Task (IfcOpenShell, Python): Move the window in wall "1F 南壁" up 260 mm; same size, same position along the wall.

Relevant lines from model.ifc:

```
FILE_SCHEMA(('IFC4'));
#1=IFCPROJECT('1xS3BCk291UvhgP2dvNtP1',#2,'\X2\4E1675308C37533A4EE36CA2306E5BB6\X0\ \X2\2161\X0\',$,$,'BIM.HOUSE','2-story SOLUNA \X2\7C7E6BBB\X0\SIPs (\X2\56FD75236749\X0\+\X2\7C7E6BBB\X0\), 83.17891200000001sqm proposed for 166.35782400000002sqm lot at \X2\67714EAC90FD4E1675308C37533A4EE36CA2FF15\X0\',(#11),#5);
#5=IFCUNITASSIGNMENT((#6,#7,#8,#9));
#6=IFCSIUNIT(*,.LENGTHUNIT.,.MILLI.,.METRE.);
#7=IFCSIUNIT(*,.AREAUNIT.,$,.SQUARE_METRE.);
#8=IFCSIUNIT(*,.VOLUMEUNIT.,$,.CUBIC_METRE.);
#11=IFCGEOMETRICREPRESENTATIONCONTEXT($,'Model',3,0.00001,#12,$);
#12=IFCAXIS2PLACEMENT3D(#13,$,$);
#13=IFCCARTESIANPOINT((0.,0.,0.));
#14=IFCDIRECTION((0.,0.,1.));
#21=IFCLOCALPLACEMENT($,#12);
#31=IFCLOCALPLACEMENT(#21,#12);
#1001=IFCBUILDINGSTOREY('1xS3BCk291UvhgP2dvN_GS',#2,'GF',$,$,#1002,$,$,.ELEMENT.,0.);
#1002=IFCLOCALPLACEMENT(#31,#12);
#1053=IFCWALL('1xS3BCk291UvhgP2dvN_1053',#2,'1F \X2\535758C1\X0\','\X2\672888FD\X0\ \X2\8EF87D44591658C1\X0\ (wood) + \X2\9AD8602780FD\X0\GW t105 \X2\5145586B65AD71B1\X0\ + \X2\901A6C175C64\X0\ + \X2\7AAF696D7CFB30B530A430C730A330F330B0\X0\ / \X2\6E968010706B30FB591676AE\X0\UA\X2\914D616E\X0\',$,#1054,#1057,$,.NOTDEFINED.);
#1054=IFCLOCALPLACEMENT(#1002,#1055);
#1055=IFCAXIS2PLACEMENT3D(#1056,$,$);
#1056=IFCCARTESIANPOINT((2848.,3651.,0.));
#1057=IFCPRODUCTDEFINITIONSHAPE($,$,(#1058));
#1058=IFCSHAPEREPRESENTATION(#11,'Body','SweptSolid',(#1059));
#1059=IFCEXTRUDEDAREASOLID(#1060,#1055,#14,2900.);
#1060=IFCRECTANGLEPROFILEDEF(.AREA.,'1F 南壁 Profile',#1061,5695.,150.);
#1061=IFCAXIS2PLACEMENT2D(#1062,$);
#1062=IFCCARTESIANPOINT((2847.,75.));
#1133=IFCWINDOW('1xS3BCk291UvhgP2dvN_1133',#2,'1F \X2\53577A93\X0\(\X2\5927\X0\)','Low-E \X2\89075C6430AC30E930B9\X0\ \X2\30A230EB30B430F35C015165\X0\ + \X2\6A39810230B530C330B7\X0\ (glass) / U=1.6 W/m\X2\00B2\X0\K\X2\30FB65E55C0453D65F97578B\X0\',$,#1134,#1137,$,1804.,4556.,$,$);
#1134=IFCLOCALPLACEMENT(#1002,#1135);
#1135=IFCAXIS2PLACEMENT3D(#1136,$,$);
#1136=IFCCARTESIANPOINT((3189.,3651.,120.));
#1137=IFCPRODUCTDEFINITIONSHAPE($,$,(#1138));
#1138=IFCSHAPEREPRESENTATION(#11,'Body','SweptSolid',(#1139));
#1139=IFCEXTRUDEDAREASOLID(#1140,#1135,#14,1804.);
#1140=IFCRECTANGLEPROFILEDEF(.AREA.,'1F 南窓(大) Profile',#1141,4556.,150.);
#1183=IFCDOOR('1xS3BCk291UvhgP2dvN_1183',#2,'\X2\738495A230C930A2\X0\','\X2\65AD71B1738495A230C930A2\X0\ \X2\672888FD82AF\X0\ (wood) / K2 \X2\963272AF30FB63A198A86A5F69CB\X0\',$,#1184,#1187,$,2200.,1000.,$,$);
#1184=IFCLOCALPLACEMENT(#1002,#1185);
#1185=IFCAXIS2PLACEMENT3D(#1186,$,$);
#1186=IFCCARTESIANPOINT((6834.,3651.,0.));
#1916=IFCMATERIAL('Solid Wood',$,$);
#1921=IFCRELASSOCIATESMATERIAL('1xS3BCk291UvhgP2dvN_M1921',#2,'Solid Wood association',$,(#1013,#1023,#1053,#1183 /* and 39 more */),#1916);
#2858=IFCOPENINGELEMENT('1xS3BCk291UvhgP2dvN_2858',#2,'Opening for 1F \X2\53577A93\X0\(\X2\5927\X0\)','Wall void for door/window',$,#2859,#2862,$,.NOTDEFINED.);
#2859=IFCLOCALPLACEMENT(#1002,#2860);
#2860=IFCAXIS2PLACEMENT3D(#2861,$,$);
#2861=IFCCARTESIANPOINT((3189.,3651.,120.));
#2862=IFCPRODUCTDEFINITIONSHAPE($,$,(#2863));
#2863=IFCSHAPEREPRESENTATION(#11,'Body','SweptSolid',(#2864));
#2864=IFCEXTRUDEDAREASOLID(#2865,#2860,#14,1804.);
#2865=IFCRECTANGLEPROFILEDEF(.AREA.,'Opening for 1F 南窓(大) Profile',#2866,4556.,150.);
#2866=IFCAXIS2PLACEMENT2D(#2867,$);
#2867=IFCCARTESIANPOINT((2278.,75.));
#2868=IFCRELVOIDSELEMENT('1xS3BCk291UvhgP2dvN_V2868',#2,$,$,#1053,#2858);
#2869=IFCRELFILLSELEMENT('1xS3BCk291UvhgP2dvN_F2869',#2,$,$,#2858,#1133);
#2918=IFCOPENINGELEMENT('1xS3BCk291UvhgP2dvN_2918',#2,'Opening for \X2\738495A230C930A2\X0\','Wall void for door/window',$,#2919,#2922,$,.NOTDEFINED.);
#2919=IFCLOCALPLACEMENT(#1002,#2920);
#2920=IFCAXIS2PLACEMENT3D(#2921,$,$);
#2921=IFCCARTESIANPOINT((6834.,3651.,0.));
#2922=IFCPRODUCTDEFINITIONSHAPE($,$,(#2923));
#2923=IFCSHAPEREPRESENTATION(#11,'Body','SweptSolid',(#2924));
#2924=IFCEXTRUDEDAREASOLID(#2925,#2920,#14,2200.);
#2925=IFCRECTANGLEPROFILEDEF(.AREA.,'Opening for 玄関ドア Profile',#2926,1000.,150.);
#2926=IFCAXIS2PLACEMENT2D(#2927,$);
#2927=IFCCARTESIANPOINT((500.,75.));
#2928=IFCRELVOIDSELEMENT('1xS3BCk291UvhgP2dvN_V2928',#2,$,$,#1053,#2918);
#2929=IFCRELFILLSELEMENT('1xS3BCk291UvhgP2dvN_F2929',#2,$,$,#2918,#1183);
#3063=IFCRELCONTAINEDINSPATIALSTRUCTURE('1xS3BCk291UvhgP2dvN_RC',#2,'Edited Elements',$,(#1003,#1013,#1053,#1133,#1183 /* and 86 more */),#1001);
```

```python
import numpy as np
import ifcopenshell
import ifcopenshell.api.geometry
import ifcopenshell.util.placement
import ifcopenshell.util.unit

model = ifcopenshell.open("model.ifc")
unit_scale = ifcopenshell.util.unit.calculate_unit_scale(model)

window = model.by_guid("1xS3BCk291UvhgP2dvN_1133")
opening = window.FillsVoids[0].RelatingOpeningElement
dz = 260.0

shift = np.array([0.0, 0.0, dz])
# The window is not placed relative to its opening, so move both.
for product in (opening, window):
    matrix = ifcopenshell.util.placement.get_local_placement(product.ObjectPlacement)
    matrix[:3, 3] += shift
    ifcopenshell.api.geometry.edit_object_placement(model, product=product, matrix=matrix, is_si=False)

print(f"moved by {dz * unit_scale:+.3f} m")

model.write("model_rev.ifc")
```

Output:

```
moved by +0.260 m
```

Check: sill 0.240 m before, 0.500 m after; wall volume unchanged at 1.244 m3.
